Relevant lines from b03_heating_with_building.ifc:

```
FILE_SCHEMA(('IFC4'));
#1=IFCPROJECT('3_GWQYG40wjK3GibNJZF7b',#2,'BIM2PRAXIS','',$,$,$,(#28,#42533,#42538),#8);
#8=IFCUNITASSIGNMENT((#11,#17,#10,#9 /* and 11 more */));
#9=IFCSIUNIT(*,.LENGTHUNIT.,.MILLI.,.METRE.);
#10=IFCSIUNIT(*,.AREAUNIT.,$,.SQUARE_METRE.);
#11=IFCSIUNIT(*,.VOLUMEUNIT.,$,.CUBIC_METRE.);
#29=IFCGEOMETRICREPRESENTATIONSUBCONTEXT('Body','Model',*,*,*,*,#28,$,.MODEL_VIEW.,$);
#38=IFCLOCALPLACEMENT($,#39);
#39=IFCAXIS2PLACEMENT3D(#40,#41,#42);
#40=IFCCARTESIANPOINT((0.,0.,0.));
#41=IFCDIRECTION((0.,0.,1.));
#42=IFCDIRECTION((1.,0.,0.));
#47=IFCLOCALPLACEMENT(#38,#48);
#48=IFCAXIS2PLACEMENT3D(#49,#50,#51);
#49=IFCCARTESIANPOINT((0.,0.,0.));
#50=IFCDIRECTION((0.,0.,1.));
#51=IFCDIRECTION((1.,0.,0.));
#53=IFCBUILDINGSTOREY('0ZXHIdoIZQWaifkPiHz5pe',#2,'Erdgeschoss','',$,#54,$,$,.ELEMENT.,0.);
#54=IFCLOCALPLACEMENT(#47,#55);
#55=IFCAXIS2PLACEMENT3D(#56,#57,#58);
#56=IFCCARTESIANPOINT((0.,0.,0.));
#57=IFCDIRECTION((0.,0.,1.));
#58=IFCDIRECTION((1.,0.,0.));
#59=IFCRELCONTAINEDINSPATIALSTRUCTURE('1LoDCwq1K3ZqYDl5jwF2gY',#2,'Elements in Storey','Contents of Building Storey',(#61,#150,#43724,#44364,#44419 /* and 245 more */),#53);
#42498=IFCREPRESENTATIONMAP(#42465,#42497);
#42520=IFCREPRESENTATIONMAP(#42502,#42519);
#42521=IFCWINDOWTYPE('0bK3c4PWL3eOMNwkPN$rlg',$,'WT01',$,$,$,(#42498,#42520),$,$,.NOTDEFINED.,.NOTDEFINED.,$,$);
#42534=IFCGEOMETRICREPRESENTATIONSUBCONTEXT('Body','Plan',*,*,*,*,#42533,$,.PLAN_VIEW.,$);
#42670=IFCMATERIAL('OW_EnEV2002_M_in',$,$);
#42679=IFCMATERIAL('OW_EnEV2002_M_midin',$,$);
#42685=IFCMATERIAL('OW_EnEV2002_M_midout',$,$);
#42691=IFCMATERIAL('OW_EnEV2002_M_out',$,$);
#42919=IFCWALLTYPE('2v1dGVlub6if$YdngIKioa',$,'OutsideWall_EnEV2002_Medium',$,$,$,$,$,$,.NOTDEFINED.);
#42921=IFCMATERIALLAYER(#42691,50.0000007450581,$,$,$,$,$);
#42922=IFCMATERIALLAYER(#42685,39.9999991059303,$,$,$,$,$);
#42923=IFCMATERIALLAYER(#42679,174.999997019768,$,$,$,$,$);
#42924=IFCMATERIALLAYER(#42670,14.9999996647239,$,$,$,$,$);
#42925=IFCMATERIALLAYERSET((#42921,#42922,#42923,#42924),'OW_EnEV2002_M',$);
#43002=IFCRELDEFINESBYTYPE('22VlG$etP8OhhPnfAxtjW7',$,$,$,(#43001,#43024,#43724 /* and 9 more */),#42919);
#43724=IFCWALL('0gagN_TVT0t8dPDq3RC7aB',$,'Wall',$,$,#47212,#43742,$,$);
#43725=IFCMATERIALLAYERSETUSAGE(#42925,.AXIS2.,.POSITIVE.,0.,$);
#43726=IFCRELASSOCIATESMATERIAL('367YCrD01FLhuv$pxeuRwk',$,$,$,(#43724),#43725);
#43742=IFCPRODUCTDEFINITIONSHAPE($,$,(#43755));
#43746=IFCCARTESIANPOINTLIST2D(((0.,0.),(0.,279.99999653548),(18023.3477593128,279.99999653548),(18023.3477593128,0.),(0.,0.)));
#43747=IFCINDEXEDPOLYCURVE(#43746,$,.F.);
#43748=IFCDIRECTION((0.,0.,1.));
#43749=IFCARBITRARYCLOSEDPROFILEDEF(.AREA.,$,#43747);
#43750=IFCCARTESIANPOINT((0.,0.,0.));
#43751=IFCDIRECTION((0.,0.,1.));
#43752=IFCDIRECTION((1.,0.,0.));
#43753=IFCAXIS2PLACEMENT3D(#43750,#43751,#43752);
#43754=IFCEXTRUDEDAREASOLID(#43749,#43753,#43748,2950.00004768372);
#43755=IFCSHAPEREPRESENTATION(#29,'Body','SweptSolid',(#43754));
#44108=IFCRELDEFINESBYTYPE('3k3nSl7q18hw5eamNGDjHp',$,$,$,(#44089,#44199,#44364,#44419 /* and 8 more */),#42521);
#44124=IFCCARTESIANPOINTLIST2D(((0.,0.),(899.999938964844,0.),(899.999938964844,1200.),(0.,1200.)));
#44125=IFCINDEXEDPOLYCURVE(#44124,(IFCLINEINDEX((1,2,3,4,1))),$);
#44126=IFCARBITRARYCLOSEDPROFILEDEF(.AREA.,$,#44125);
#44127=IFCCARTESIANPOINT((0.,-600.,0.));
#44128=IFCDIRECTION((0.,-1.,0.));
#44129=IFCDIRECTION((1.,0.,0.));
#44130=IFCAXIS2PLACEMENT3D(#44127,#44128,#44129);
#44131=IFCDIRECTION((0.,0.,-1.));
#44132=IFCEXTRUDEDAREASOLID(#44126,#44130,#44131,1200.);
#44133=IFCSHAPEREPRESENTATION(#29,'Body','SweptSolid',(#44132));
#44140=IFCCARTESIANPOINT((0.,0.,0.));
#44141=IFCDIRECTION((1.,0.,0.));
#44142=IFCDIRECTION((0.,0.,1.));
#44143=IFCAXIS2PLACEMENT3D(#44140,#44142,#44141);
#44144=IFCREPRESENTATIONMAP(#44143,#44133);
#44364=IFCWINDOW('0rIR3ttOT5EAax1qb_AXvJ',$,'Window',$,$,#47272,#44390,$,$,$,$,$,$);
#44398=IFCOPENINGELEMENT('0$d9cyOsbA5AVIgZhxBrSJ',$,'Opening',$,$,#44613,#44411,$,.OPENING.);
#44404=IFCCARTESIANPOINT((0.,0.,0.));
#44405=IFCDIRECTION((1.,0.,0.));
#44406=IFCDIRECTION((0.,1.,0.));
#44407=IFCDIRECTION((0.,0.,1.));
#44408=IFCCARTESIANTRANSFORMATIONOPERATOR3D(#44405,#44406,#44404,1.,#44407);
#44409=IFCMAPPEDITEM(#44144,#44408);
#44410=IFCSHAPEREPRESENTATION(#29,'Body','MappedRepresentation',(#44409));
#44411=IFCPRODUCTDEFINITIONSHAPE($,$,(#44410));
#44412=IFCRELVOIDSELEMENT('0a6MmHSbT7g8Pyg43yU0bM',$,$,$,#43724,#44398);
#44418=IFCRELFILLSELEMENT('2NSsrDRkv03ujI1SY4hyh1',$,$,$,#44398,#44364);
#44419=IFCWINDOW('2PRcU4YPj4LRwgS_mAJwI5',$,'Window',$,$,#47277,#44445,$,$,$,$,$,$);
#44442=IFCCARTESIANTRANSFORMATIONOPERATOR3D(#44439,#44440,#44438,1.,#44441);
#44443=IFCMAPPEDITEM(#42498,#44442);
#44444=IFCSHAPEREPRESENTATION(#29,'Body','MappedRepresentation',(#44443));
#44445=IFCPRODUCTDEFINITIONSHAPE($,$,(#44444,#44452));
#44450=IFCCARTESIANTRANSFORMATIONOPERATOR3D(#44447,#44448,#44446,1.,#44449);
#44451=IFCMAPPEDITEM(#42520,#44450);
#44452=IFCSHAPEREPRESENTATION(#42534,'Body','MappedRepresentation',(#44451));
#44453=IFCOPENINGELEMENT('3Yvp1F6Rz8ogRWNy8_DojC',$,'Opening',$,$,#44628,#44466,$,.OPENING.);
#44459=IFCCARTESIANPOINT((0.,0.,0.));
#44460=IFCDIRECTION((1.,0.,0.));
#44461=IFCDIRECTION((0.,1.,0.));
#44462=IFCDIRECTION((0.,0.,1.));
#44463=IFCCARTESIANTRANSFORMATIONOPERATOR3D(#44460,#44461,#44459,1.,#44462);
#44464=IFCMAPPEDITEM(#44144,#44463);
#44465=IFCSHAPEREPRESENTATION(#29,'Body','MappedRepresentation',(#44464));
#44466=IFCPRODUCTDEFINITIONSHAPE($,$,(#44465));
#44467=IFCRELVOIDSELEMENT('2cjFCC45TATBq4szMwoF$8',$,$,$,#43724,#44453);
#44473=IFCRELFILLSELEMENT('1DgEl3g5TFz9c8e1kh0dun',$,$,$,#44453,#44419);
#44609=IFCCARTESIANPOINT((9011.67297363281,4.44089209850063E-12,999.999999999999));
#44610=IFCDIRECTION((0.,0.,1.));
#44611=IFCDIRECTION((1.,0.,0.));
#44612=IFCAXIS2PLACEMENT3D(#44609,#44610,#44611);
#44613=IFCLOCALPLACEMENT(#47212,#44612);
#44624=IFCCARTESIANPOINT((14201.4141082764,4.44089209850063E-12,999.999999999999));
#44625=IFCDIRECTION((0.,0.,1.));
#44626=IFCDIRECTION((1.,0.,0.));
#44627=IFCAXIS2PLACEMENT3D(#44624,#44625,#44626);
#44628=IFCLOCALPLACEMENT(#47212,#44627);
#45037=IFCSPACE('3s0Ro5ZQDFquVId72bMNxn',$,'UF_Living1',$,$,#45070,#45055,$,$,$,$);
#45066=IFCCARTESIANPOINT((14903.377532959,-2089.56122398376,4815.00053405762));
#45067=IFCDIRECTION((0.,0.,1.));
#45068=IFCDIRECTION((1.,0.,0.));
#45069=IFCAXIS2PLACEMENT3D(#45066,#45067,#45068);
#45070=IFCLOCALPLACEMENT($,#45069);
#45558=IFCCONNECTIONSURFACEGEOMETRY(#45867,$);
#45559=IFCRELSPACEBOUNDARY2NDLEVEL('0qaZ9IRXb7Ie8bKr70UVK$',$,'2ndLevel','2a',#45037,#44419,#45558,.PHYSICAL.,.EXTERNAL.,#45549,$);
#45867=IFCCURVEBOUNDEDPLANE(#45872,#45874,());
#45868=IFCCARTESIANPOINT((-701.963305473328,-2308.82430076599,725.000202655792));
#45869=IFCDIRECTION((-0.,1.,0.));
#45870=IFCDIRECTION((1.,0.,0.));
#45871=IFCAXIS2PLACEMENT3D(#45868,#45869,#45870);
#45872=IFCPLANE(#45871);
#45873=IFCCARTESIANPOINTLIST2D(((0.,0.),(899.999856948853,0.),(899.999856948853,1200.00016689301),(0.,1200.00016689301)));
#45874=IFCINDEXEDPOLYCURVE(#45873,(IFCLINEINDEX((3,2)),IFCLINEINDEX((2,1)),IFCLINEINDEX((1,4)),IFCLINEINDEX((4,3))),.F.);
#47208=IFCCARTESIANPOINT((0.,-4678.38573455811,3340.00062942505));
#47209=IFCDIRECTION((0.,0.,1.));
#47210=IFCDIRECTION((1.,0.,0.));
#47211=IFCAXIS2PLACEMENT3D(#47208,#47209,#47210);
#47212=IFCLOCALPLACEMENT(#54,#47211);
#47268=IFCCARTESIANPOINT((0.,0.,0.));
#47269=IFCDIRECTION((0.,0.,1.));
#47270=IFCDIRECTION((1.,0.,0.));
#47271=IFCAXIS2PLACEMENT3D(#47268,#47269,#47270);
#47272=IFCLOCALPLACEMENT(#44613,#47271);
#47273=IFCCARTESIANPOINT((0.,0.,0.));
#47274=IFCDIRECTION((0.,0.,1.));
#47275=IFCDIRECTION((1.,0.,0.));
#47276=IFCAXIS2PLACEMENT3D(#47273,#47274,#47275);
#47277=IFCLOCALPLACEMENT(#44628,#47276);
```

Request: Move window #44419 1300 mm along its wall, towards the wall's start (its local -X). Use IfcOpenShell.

```python
import numpy as np
import ifcopenshell
import ifcopenshell.api.geometry
import ifcopenshell.util.placement
import ifcopenshell.util.unit

model = ifcopenshell.open("b03_heating_with_building.ifc")
unit_scale = ifcopenshell.util.unit.calculate_unit_scale(model)

window = model.by_guid("2PRcU4YPj4LRwgS_mAJwI5")
opening = window.FillsVoids[0].RelatingOpeningElement
wall = opening.VoidsElements[0].RelatingBuildingElement

wall_matrix = ifcopenshell.util.placement.get_local_placement(wall.ObjectPlacement)
shift = wall_matrix[:3, 0] * -1.3 / unit_scale
before = ifcopenshell.util.placement.get_local_placement(window.ObjectPlacement)[:3, 3].copy()

# The window is placed relative to its opening, so it follows when the opening moves.
matrix = ifcopenshell.util.placement.get_local_placement(opening.ObjectPlacement)
matrix[:3, 3] += shift
ifcopenshell.api.geometry.edit_object_placement(
    model, product=opening, matrix=matrix, is_si=False, should_transform_children=True
)

# Space boundary surfaces are stored in each space's coordinates; move them too.
for rel in window.ProvidesBoundaries:
    if not rel.ConnectionGeometry:
        continue
    surface = rel.ConnectionGeometry.SurfaceOnRelatingElement.BasisSurface
    space_matrix = ifcopenshell.util.placement.get_local_placement(rel.RelatingSpace.ObjectPlacement)
    point = np.array(surface.Position.Location.Coordinates) + space_matrix[:3, :3].T @ shift
    surface.Position = model.createIfcAxis2Placement3D(
        model.createIfcCartesianPoint(point.tolist()), surface.Position.Axis, surface.Position.RefDirection
    )

after = ifcopenshell.util.placement.get_local_placement(window.ObjectPlacement)[:3, 3]
print("window moved by", (after - before).round(3) + 0.0)

model.write("b03_heating_with_building_updated.ifc")
```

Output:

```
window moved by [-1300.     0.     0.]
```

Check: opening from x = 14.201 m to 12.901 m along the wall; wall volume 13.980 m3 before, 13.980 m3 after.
